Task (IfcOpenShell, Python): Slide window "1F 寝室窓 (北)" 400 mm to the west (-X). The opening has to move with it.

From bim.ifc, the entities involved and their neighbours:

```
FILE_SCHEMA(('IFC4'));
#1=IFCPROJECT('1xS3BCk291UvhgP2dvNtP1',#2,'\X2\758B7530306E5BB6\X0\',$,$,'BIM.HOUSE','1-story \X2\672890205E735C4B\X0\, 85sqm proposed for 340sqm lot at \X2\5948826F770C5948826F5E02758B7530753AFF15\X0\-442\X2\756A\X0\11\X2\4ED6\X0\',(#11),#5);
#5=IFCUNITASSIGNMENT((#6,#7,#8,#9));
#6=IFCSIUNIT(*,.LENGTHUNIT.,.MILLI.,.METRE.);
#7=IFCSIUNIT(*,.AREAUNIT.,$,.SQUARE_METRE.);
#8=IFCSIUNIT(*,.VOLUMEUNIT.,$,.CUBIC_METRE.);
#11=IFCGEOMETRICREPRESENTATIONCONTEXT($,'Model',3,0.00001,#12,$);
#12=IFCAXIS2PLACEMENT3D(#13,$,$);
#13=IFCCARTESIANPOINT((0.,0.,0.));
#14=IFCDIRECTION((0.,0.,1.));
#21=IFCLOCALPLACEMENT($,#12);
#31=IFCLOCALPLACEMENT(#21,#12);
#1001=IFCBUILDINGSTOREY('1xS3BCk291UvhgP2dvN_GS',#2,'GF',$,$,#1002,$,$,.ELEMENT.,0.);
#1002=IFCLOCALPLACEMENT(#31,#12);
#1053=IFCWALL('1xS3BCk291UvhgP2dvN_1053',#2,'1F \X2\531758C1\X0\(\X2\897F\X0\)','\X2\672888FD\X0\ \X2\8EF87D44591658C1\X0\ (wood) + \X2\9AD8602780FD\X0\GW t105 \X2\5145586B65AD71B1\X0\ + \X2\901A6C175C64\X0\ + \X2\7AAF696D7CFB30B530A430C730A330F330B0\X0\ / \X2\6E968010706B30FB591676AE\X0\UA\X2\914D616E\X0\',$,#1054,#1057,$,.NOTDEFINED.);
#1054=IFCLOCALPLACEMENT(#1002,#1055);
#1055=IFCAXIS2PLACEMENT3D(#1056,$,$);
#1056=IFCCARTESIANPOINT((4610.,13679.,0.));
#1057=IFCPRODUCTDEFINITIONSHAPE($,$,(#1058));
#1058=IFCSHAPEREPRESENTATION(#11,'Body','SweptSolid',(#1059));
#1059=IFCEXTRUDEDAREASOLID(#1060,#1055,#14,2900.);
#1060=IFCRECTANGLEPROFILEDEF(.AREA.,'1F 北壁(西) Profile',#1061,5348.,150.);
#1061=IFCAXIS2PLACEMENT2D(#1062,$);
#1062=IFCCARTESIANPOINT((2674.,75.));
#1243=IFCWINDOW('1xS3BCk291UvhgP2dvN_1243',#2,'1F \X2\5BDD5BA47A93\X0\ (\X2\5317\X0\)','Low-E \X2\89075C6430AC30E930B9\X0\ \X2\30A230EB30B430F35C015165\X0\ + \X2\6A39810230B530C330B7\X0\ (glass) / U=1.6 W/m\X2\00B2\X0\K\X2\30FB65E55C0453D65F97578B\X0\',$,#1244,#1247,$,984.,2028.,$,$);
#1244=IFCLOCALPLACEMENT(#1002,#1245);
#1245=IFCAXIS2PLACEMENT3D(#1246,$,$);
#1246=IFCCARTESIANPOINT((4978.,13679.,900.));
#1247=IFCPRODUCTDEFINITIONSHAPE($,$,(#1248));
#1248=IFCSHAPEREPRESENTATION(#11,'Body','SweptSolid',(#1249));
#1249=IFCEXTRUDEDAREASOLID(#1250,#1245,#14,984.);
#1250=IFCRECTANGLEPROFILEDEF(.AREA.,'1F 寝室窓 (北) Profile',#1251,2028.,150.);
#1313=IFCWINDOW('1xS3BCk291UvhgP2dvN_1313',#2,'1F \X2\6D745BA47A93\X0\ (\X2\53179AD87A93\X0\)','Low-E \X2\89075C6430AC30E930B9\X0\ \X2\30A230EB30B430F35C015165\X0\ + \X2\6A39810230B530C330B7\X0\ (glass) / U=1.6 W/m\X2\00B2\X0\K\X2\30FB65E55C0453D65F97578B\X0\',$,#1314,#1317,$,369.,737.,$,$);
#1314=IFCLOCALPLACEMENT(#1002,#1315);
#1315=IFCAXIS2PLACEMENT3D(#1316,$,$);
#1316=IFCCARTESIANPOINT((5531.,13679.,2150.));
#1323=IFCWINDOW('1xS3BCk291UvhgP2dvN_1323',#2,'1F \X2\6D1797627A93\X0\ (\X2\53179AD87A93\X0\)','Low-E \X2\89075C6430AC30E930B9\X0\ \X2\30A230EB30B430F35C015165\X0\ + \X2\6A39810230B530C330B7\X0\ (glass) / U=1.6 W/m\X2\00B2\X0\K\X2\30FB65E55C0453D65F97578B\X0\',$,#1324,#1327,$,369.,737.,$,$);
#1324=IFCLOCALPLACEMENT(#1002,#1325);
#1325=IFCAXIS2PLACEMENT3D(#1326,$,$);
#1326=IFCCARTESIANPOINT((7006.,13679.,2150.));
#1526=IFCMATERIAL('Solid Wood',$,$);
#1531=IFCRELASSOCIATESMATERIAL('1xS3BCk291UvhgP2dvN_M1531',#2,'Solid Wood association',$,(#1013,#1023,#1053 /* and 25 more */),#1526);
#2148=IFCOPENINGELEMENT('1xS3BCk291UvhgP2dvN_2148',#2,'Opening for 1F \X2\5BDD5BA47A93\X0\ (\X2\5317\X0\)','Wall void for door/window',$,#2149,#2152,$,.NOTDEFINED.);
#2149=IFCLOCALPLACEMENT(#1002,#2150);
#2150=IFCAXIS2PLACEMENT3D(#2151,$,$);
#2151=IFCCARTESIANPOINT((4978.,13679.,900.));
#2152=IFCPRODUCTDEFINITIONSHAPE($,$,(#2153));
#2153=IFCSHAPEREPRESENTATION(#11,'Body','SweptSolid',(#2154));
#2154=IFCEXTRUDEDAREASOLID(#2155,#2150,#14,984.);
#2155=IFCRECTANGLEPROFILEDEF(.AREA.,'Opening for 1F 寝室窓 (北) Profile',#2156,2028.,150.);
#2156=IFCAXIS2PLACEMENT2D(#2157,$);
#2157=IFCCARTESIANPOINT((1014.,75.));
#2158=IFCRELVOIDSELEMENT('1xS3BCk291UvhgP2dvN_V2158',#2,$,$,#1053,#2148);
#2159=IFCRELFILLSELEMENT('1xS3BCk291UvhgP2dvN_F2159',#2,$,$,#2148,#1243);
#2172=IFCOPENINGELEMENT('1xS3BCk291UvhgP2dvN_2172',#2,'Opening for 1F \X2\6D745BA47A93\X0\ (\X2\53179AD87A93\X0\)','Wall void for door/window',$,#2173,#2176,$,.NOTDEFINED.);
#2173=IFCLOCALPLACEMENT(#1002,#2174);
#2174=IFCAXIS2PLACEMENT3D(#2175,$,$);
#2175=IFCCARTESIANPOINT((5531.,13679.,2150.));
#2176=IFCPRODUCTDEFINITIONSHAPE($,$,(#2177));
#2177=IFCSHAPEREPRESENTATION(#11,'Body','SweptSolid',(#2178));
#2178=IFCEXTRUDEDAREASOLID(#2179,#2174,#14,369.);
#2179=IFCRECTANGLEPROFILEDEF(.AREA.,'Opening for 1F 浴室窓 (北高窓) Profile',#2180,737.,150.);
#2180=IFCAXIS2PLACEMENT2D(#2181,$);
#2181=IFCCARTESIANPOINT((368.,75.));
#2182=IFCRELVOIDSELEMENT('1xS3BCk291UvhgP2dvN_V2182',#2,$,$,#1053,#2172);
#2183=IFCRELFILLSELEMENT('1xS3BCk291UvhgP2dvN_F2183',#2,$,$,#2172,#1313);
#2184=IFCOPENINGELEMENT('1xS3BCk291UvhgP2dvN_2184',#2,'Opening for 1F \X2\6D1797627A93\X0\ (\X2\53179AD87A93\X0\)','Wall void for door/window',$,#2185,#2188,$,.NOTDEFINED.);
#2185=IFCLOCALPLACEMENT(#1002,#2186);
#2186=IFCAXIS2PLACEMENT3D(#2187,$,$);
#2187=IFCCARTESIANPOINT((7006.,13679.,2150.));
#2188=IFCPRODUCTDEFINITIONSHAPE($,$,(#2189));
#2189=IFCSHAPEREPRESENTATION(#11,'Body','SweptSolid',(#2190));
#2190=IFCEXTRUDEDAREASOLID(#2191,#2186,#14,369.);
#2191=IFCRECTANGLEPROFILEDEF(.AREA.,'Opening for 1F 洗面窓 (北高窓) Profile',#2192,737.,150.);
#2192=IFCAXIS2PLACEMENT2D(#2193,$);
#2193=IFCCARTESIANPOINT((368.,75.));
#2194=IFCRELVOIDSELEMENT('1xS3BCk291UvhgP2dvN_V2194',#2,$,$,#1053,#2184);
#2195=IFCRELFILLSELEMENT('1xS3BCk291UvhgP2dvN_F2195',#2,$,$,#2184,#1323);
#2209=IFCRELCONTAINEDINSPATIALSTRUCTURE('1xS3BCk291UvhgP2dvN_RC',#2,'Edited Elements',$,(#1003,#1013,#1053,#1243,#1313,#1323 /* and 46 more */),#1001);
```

```python
import ifcopenshell
import ifcopenshell.api.geometry
import ifcopenshell.util.placement

model = ifcopenshell.open("bim.ifc")

window = model.by_guid("1xS3BCk291UvhgP2dvN_1243")
opening = window.FillsVoids[0].RelatingOpeningElement
wall = opening.VoidsElements[0].RelatingBuildingElement

wall_matrix = ifcopenshell.util.placement.get_local_placement(wall.ObjectPlacement)
shift = wall_matrix[:3, 0] * -400.0
before = ifcopenshell.util.placement.get_local_placement(window.ObjectPlacement)[:3, 3].copy()

# The window is not placed relative to its opening, so move both.
for product in (opening, window):
    matrix = ifcopenshell.util.placement.get_local_placement(product.ObjectPlacement)
    matrix[:3, 3] += shift
    ifcopenshell.api.geometry.edit_object_placement(model, product=product, matrix=matrix, is_si=False)

after = ifcopenshell.util.placement.get_local_placement(window.ObjectPlacement)[:3, 3]
print("window moved by", (after - before).round(3) + 0.0)

model.write("bim_updated.ifc")
```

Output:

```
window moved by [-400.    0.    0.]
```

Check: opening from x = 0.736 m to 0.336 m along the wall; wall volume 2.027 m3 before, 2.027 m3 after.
